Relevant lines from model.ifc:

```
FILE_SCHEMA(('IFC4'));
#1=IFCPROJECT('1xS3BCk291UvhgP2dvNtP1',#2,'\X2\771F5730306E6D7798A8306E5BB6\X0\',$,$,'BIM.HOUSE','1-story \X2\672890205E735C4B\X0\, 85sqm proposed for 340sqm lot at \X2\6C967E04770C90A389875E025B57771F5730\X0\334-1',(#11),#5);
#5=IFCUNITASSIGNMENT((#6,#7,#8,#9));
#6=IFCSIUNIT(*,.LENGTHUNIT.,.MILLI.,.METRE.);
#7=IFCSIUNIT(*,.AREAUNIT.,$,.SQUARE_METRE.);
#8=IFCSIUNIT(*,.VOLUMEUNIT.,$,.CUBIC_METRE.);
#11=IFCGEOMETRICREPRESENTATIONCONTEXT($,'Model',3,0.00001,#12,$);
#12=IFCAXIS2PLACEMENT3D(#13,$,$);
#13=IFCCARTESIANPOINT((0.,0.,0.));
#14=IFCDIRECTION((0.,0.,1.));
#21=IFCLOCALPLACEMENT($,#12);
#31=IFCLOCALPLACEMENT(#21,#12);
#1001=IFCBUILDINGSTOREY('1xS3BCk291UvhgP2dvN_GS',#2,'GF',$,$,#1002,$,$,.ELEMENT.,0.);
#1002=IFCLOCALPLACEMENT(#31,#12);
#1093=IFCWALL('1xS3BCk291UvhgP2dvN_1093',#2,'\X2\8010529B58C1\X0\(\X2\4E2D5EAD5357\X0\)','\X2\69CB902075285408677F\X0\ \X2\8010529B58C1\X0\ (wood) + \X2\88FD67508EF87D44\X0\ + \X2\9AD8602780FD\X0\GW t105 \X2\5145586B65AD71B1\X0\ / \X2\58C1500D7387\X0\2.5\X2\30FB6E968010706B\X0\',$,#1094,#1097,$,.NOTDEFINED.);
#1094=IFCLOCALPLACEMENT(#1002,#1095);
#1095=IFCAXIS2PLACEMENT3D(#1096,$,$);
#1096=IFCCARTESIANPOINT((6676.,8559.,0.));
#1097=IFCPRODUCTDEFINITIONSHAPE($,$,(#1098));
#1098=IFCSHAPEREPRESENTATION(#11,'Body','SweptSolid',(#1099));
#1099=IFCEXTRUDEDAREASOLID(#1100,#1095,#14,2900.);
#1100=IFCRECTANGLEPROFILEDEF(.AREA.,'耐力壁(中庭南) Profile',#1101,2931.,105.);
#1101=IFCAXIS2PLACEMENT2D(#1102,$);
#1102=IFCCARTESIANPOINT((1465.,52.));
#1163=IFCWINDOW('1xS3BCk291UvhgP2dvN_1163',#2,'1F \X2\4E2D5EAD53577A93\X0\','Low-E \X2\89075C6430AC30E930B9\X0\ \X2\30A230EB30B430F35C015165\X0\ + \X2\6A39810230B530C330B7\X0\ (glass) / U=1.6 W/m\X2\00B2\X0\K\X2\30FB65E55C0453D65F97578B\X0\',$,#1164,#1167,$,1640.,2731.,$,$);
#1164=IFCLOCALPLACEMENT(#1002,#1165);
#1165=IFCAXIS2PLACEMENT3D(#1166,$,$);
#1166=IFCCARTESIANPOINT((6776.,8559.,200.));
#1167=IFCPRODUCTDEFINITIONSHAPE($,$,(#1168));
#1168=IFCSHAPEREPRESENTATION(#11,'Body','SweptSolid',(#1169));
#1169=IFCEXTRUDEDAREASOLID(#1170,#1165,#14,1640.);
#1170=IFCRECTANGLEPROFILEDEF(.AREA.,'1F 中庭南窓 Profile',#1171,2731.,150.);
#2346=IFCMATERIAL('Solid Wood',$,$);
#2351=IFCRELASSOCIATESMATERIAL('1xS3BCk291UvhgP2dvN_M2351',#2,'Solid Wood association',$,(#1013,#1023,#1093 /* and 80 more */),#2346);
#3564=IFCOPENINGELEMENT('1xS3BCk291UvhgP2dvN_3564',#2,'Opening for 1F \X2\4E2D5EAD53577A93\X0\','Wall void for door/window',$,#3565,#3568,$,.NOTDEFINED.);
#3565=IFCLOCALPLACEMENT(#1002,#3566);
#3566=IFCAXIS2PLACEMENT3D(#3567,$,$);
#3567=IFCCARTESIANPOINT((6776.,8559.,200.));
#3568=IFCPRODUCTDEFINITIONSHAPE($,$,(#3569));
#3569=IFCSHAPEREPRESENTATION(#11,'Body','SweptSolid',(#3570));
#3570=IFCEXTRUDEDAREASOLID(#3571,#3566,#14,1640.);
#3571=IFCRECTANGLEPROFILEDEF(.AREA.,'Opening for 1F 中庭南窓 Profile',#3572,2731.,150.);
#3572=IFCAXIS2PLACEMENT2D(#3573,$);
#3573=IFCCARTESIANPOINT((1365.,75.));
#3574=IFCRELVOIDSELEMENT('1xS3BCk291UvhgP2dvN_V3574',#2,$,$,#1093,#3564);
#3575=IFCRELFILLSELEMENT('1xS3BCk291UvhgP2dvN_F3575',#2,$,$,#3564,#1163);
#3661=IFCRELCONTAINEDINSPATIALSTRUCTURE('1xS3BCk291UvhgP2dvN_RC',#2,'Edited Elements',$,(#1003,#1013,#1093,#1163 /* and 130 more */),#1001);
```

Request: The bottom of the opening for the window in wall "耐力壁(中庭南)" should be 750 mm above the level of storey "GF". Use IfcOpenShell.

```python
import numpy as np
import ifcopenshell
import ifcopenshell.api.geometry
import ifcopenshell.geom
import ifcopenshell.util.element
import ifcopenshell.util.placement
import ifcopenshell.util.shape
import ifcopenshell.util.unit

model = ifcopenshell.open("model.ifc")
unit_scale = ifcopenshell.util.unit.calculate_unit_scale(model)

window = model.by_guid("1xS3BCk291UvhgP2dvN_1163")
opening = window.FillsVoids[0].RelatingOpeningElement
storey = ifcopenshell.util.element.get_container(window, ifc_class="IfcBuildingStorey")
level = ifcopenshell.util.placement.get_local_placement(storey.ObjectPlacement)[2, 3]

# The opening's origin need not be at the sill, so measure its lowest point.
shape = ifcopenshell.geom.create_shape(ifcopenshell.geom.settings(), opening)
bottom = ifcopenshell.util.shape.get_shape_bottom_elevation(shape, shape.geometry) / unit_scale
dz = level + 0.75 / unit_scale - bottom

shift = np.array([0.0, 0.0, dz])
# The window is not placed relative to its opening, so move both.
for product in (opening, window):
    matrix = ifcopenshell.util.placement.get_local_placement(product.ObjectPlacement)
    matrix[:3, 3] += shift
    ifcopenshell.api.geometry.edit_object_placement(model, product=product, matrix=matrix, is_si=False)

print(f"moved by {dz * unit_scale:+.3f} m")

model.write("model-out.ifc")
```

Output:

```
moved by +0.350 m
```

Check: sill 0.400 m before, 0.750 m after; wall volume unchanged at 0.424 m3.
